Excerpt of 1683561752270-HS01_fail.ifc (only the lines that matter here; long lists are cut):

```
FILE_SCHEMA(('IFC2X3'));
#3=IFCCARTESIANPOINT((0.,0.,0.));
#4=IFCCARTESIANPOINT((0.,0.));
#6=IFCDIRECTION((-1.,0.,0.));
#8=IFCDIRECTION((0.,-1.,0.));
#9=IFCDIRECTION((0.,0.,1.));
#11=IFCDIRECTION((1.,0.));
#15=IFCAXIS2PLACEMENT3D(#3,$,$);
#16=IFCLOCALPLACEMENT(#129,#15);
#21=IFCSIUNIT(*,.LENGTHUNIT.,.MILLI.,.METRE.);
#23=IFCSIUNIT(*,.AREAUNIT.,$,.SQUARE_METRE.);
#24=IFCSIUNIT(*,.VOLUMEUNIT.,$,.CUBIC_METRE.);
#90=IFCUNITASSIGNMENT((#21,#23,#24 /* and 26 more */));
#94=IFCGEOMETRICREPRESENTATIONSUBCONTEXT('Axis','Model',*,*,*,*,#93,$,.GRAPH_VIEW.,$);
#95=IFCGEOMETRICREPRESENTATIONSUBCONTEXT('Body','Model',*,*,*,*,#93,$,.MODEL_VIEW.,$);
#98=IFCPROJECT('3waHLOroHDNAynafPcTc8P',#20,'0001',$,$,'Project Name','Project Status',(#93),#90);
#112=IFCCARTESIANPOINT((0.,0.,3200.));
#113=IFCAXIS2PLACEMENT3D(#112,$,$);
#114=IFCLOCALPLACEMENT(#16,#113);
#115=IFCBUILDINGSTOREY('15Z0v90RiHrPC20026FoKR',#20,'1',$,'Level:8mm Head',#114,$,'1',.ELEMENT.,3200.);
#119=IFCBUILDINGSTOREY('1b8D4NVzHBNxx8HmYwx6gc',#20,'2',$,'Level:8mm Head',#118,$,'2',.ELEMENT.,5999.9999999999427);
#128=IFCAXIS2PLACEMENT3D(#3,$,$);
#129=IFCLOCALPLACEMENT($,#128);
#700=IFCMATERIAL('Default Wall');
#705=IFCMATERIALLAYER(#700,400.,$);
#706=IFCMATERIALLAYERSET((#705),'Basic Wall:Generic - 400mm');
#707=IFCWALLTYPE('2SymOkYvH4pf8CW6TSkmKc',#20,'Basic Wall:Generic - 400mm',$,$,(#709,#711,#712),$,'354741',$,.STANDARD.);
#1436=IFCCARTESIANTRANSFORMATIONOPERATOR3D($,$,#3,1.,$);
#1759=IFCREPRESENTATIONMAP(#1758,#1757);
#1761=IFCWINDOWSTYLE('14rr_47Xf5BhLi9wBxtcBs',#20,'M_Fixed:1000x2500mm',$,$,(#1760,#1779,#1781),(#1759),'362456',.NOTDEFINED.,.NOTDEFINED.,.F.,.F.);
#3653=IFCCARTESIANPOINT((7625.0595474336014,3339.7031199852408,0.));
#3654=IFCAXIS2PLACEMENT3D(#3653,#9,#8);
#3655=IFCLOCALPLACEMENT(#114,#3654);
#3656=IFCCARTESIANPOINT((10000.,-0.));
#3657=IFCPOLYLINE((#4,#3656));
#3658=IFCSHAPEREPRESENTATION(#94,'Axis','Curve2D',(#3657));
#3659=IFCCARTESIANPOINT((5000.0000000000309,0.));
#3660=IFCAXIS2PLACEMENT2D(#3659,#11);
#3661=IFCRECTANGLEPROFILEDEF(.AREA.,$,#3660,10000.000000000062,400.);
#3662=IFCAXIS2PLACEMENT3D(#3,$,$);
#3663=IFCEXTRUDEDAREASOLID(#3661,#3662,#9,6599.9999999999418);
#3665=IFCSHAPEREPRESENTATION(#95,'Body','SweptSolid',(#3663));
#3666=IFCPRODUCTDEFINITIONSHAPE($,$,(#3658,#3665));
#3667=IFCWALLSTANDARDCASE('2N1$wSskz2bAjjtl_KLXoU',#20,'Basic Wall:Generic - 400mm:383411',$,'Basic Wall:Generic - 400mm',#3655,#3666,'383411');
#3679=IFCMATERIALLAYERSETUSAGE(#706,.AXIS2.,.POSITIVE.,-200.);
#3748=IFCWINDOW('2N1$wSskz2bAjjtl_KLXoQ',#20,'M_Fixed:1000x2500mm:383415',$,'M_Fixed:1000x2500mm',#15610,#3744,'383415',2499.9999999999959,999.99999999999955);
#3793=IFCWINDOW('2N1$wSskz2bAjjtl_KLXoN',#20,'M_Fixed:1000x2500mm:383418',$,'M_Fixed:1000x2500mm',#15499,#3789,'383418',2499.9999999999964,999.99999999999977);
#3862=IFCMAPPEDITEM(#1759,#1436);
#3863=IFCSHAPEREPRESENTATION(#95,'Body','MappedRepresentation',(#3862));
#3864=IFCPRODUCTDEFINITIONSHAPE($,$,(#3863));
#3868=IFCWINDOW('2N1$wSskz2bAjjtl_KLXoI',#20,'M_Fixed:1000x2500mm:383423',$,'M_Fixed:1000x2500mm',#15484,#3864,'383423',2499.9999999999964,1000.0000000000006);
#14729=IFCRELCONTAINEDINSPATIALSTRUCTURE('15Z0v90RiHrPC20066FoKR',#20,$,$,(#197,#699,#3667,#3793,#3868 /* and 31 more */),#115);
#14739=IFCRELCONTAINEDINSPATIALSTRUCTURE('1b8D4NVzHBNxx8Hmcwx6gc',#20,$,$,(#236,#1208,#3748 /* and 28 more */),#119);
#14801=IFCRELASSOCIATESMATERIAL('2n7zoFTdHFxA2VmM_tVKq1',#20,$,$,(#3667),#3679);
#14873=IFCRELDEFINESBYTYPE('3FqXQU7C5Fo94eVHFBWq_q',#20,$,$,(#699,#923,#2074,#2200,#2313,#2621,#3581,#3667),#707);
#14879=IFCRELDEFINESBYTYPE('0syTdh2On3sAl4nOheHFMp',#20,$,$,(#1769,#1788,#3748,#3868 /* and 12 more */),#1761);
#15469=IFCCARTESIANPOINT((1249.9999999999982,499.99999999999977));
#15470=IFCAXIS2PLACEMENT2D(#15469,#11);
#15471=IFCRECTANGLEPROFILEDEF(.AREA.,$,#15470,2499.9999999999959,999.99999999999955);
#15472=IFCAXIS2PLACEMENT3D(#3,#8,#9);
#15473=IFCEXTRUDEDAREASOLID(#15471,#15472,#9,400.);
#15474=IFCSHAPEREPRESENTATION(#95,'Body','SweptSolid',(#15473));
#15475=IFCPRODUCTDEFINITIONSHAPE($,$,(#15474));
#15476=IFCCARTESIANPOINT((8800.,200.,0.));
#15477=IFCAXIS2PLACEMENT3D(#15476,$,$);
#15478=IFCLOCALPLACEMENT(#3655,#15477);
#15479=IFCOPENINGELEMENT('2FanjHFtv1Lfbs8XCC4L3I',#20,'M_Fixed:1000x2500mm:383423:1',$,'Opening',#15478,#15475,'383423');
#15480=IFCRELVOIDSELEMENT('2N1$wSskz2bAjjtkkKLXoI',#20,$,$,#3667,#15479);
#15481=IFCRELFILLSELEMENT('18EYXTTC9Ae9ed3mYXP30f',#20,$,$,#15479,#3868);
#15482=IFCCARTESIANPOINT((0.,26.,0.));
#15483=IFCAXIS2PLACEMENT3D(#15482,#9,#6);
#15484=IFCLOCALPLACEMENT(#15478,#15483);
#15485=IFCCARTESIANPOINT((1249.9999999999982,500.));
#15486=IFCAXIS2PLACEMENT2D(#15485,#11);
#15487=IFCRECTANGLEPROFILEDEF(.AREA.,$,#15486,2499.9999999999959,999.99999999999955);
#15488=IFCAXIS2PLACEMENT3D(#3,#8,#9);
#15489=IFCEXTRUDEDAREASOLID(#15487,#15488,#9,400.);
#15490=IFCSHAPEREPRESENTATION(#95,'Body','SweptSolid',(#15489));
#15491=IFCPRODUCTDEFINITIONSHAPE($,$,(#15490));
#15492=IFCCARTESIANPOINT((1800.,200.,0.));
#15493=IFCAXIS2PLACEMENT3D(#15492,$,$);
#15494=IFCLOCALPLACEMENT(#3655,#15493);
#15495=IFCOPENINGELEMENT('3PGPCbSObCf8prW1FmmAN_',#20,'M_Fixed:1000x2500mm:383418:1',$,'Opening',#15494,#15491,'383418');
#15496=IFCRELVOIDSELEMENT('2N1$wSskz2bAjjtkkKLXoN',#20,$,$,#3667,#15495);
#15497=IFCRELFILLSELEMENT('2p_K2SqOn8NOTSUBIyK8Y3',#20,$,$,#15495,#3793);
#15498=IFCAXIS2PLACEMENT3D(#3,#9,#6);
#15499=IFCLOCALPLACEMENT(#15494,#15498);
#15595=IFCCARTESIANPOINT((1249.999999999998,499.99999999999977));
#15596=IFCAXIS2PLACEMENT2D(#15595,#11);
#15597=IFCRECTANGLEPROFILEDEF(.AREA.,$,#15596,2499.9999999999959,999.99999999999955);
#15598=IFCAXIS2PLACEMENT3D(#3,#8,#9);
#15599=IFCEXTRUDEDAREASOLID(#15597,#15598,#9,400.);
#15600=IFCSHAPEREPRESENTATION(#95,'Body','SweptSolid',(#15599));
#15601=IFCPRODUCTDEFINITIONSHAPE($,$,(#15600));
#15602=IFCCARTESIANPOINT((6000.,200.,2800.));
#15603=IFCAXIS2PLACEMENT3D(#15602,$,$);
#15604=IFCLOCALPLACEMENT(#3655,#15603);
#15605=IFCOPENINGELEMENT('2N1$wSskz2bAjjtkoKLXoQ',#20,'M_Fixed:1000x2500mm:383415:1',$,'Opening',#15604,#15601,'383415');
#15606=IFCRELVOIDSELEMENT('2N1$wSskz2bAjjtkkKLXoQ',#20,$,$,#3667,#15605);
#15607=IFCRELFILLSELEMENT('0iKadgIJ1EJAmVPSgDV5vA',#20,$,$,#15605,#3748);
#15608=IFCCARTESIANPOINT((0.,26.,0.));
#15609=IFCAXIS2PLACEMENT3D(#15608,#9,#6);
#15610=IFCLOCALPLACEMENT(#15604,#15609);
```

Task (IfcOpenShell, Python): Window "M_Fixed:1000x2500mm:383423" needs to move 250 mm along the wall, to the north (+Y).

```python
import ifcopenshell
import ifcopenshell.api.geometry
import ifcopenshell.util.placement
import ifcopenshell.util.unit

model = ifcopenshell.open("1683561752270-HS01_fail.ifc")
unit_scale = ifcopenshell.util.unit.calculate_unit_scale(model)

window = model.by_guid("2N1$wSskz2bAjjtl_KLXoI")
opening = window.FillsVoids[0].RelatingOpeningElement
wall = opening.VoidsElements[0].RelatingBuildingElement

wall_matrix = ifcopenshell.util.placement.get_local_placement(wall.ObjectPlacement)
shift = wall_matrix[:3, 0] * -0.25 / unit_scale
before = ifcopenshell.util.placement.get_local_placement(window.ObjectPlacement)[:3, 3].copy()

# The window is placed relative to its opening, so it follows when the opening moves.
matrix = ifcopenshell.util.placement.get_local_placement(opening.ObjectPlacement)
matrix[:3, 3] += shift
ifcopenshell.api.geometry.edit_object_placement(
    model, product=opening, matrix=matrix, is_si=False, should_transform_children=True
)

after = ifcopenshell.util.placement.get_local_placement(window.ObjectPlacement)[:3, 3]
print("window moved by", (after - before).round(3) + 0.0)

model.write("1683561752270-HS01_fail_edited.ifc")
```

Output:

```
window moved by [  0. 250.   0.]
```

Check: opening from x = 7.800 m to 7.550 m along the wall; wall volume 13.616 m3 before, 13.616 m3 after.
